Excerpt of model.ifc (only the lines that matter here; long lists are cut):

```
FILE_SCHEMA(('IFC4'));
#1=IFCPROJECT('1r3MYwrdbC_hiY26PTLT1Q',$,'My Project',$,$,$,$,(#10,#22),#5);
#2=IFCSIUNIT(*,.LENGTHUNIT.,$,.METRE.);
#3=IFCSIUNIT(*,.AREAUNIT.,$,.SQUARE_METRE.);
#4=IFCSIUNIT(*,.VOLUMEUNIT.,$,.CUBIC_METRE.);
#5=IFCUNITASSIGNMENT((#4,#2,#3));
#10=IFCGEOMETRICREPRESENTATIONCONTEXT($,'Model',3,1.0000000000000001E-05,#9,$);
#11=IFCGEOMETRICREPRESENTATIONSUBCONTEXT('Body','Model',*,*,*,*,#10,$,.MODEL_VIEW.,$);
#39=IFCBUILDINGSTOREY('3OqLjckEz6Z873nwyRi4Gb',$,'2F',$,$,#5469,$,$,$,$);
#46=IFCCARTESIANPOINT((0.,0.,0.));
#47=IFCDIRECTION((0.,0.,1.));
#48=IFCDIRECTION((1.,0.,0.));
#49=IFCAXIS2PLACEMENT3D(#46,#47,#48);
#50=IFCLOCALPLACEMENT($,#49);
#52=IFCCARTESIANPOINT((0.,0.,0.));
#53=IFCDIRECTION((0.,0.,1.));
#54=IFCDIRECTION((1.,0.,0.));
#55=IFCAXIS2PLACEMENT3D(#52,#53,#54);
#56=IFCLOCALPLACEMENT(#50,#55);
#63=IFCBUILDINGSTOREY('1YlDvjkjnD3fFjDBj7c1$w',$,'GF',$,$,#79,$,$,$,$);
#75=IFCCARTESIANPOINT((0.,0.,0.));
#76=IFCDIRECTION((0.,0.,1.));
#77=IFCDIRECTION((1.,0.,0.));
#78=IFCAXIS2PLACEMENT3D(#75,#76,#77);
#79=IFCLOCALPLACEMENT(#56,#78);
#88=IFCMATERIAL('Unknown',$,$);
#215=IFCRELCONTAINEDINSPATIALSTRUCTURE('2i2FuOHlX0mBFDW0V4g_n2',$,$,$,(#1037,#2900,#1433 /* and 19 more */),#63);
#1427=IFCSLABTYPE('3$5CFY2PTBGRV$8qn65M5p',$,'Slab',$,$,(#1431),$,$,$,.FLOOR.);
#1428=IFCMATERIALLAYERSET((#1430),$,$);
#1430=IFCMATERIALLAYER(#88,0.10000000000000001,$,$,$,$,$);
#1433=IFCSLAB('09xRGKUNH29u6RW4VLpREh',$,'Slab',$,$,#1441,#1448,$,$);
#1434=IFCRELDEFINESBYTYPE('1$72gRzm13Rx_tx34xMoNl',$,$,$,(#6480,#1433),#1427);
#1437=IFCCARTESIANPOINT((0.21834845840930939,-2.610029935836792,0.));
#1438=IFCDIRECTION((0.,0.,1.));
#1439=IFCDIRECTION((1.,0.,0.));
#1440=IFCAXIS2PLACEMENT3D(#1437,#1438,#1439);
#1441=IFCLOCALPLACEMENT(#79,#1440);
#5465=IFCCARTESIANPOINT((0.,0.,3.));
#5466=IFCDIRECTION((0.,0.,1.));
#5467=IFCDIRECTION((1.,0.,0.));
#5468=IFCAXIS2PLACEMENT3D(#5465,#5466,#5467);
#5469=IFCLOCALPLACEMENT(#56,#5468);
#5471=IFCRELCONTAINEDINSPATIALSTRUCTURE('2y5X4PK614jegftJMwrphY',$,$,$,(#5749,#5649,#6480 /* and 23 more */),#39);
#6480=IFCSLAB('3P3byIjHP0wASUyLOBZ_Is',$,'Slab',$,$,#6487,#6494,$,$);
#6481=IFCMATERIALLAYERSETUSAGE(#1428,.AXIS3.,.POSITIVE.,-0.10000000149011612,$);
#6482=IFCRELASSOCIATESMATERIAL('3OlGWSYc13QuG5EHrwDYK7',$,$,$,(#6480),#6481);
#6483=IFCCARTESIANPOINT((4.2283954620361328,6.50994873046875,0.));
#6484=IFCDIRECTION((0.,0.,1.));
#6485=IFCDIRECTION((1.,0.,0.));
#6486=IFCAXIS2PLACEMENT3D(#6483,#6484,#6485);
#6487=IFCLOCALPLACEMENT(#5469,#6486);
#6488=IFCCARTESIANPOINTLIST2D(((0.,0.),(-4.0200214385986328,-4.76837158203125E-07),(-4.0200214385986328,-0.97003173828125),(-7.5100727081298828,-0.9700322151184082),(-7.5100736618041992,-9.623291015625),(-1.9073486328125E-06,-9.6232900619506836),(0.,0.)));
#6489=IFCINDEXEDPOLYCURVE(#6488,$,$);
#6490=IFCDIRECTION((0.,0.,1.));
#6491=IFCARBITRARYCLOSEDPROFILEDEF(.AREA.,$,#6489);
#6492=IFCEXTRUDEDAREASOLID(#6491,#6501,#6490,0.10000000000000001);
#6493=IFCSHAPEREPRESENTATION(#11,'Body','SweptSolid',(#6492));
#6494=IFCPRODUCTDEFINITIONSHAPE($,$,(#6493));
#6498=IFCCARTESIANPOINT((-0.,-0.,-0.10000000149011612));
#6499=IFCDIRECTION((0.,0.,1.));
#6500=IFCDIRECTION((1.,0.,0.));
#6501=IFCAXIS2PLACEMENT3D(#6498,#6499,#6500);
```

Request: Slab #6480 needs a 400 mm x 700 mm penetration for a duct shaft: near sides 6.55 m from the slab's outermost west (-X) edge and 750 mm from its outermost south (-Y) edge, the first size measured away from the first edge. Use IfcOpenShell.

```python
import numpy as np
import ifcopenshell
import ifcopenshell.api.feature
import ifcopenshell.api.geometry
import ifcopenshell.api.root
import ifcopenshell.geom
import ifcopenshell.util.placement
import ifcopenshell.util.representation
import ifcopenshell.util.shape
import ifcopenshell.util.unit

model = ifcopenshell.open("model.ifc")
unit_scale = ifcopenshell.util.unit.calculate_unit_scale(model)
settings = ifcopenshell.geom.settings()


def volume(element):
    """Net volume in cubic metres, openings subtracted."""
    shape = ifcopenshell.geom.create_shape(settings, element)
    return ifcopenshell.util.shape.get_volume(shape.geometry)


slab = model.by_guid("3P3byIjHP0wASUyLOBZ_Is")
before = volume(slab)

# Extent in the slab's own axes, in metres. The edges named are its -X and -Y sides.
slab_shape = ifcopenshell.geom.create_shape(settings, slab)
vertices = ifcopenshell.util.shape.get_vertices(slab_shape.geometry)
x_min, y_min, bottom = vertices.min(axis=0)
top = vertices[:, 2].max()

opening = ifcopenshell.api.root.create_entity(model, ifc_class="IfcOpeningElement", name="Duct shaft opening", predefined_type="OPENING")
context = ifcopenshell.util.representation.get_context(model, "Model", "Body", "MODEL_VIEW")
width, depth = 0.4, 0.7
outline = [(0.0, 0.0), (width, 0.0), (width, depth), (0.0, depth), (0.0, 0.0)]
# Overshoot both faces by 50 mm so the cut is clean.
shape = ifcopenshell.api.geometry.add_slab_representation(
    model, context=context, depth=top - bottom + 0.1, polyline=outline
)
ifcopenshell.api.geometry.assign_representation(model, product=opening, representation=shape)

matrix = ifcopenshell.util.placement.get_local_placement(slab.ObjectPlacement)
matrix[:, 3] = matrix @ np.append(np.array([x_min + 6.55, y_min + 0.75, bottom - 0.05]) / unit_scale, 1.0)
ifcopenshell.api.geometry.edit_object_placement(model, product=opening, matrix=matrix, is_si=False)
ifcopenshell.api.feature.add_feature(model, feature=opening, element=slab)

after = volume(slab)

print(f"slab volume {before:.3f} -> {after:.3f} m3")

model.write("model_edited.ifc")
```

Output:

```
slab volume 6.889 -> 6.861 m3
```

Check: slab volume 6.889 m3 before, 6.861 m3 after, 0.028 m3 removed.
